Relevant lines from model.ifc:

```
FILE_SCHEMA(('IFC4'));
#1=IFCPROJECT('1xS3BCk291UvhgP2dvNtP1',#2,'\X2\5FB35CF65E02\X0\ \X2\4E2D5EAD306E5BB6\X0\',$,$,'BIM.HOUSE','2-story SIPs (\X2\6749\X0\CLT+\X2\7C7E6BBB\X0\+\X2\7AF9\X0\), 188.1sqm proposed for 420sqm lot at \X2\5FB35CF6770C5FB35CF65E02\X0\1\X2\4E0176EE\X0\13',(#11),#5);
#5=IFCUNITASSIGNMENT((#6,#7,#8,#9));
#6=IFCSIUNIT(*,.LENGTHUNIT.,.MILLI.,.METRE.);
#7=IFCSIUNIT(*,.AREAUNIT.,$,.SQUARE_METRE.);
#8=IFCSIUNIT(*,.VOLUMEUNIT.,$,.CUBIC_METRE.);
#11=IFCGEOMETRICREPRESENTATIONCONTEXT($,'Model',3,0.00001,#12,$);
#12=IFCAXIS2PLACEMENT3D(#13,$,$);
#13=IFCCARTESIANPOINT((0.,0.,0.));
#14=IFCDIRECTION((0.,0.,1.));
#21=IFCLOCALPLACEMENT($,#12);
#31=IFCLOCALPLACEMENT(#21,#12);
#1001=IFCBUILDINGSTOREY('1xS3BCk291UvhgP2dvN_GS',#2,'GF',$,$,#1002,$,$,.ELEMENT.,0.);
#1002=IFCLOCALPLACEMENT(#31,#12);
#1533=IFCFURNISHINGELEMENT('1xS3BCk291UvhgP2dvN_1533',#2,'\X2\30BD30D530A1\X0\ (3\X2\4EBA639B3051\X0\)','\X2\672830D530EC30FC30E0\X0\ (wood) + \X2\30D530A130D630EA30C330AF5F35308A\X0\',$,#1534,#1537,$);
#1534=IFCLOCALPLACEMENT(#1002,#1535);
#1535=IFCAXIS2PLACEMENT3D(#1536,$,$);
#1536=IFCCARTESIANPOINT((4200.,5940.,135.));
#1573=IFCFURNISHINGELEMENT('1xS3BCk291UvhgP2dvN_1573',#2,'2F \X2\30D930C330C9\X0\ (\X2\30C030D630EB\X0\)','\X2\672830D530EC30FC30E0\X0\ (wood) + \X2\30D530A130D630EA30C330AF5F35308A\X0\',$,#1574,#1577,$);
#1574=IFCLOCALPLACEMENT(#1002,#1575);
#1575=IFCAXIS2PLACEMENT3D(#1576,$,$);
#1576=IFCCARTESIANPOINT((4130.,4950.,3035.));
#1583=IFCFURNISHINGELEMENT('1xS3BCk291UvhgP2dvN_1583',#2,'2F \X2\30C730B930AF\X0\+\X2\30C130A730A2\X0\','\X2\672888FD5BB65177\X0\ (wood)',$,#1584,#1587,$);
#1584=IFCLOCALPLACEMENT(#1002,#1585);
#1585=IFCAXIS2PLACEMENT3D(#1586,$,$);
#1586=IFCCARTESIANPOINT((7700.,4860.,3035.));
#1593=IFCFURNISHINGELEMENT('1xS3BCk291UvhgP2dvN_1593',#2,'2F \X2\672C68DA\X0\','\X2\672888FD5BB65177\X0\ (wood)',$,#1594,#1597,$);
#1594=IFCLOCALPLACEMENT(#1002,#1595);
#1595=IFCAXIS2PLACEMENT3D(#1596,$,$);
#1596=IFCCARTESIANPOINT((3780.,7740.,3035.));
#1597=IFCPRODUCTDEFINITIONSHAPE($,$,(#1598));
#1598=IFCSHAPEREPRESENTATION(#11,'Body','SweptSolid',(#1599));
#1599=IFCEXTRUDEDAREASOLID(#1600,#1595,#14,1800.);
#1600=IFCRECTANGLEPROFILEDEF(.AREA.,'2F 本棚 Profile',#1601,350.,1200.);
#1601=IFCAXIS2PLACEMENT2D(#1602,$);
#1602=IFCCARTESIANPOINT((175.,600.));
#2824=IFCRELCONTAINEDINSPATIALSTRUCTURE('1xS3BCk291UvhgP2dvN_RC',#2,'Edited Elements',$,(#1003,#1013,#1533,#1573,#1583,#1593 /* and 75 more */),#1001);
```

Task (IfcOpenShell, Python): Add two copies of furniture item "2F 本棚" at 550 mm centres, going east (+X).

```python
import numpy as np
import ifcopenshell
import ifcopenshell.api.geometry
import ifcopenshell.api.root
import ifcopenshell.util.element
import ifcopenshell.util.placement
import ifcopenshell.util.unit

model = ifcopenshell.open("model.ifc")
unit_scale = ifcopenshell.util.unit.calculate_unit_scale(model)


def reuse_history(source, copy):
    """copy_class also copies each property set's owner history, people and application; keep the originals."""
    for rel in copy.IsDefinedBy:
        if rel.is_a("IfcRelDefinesByProperties") and (history := rel.RelatingPropertyDefinition.OwnerHistory):
            rel.RelatingPropertyDefinition.OwnerHistory = source.OwnerHistory
            ifcopenshell.util.element.remove_deep2(model, history)


source = model.by_guid("1xS3BCk291UvhgP2dvN_1593")
base = ifcopenshell.util.placement.get_local_placement(source.ObjectPlacement)
step = np.array([1.0, 0.0, 0.0]) * 0.55 / unit_scale

for i in range(1, 3):
    copy = ifcopenshell.api.root.copy_class(model, product=source)
    copy.Representation = ifcopenshell.util.element.copy_deep(
        model, source.Representation, exclude=["IfcGeometricRepresentationContext", "IfcRepresentationMap"]
    )
    reuse_history(source, copy)
    matrix = base.copy()
    matrix[:3, 3] += i * step
    print("added at", matrix[:3, 3].round(3) + 0.0)
    ifcopenshell.api.geometry.edit_object_placement(model, product=copy, matrix=matrix, is_si=False)

model.write("model-out.ifc")
```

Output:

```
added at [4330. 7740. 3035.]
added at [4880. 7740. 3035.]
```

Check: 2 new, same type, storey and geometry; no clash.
